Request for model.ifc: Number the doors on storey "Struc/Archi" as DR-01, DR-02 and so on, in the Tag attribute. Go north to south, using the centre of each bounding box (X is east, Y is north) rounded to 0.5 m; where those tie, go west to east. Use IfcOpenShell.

First a look at what the model holds.

```python
import ifcopenshell
import ifcopenshell.util.element
import ifcopenshell.util.placement

model = ifcopenshell.open("model.ifc")
print(model.schema)
storey = next(s for s in model.by_type("IfcBuildingStorey") if s.Name == "Struc/Archi")
doors = [e for e in ifcopenshell.util.element.get_decomposition(storey) if e.is_a("IfcDoor")]
for e in sorted(doors, key=lambda e: e.id()):
    origin = ifcopenshell.util.placement.get_local_placement(e.ObjectPlacement)[:3, 3]
    print(e.id(), e.Tag, e.Name, origin.round(2) + 0.0, sep=" | ")
```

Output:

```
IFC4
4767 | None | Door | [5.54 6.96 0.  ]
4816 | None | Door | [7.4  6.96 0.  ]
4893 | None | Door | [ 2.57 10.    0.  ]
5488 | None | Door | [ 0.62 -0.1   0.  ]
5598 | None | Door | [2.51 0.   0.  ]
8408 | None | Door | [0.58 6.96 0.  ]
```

```python
import ifcopenshell
import ifcopenshell.geom
import ifcopenshell.util.element
import ifcopenshell.util.shape

model = ifcopenshell.open("model.ifc")
settings = ifcopenshell.geom.settings()
settings.set("use-world-coords", True)


def centre(element):
    shape = ifcopenshell.geom.create_shape(settings, element)
    return ifcopenshell.util.shape.get_bbox_centroid(shape.geometry)


storey = next(s for s in model.by_type("IfcBuildingStorey") if s.Name == "Struc/Archi")
doors = [e for e in ifcopenshell.util.element.get_decomposition(storey) if e.is_a("IfcDoor")]

# Insertion points can sit at a corner or the storey origin, so sort by the geometry (in metres).
centres = {e: centre(e) for e in doors}
doors.sort(key=lambda e: (-round(centres[e][1] / 0.5), centres[e][0]))

for i, e in enumerate(doors, start=1):
    number = f"DR-{i:02d}"
    e.Tag = number
    print(e.id(), number)

model.write("model_rev.ifc")
```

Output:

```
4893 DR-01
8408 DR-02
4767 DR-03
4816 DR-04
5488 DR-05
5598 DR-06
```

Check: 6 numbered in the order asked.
